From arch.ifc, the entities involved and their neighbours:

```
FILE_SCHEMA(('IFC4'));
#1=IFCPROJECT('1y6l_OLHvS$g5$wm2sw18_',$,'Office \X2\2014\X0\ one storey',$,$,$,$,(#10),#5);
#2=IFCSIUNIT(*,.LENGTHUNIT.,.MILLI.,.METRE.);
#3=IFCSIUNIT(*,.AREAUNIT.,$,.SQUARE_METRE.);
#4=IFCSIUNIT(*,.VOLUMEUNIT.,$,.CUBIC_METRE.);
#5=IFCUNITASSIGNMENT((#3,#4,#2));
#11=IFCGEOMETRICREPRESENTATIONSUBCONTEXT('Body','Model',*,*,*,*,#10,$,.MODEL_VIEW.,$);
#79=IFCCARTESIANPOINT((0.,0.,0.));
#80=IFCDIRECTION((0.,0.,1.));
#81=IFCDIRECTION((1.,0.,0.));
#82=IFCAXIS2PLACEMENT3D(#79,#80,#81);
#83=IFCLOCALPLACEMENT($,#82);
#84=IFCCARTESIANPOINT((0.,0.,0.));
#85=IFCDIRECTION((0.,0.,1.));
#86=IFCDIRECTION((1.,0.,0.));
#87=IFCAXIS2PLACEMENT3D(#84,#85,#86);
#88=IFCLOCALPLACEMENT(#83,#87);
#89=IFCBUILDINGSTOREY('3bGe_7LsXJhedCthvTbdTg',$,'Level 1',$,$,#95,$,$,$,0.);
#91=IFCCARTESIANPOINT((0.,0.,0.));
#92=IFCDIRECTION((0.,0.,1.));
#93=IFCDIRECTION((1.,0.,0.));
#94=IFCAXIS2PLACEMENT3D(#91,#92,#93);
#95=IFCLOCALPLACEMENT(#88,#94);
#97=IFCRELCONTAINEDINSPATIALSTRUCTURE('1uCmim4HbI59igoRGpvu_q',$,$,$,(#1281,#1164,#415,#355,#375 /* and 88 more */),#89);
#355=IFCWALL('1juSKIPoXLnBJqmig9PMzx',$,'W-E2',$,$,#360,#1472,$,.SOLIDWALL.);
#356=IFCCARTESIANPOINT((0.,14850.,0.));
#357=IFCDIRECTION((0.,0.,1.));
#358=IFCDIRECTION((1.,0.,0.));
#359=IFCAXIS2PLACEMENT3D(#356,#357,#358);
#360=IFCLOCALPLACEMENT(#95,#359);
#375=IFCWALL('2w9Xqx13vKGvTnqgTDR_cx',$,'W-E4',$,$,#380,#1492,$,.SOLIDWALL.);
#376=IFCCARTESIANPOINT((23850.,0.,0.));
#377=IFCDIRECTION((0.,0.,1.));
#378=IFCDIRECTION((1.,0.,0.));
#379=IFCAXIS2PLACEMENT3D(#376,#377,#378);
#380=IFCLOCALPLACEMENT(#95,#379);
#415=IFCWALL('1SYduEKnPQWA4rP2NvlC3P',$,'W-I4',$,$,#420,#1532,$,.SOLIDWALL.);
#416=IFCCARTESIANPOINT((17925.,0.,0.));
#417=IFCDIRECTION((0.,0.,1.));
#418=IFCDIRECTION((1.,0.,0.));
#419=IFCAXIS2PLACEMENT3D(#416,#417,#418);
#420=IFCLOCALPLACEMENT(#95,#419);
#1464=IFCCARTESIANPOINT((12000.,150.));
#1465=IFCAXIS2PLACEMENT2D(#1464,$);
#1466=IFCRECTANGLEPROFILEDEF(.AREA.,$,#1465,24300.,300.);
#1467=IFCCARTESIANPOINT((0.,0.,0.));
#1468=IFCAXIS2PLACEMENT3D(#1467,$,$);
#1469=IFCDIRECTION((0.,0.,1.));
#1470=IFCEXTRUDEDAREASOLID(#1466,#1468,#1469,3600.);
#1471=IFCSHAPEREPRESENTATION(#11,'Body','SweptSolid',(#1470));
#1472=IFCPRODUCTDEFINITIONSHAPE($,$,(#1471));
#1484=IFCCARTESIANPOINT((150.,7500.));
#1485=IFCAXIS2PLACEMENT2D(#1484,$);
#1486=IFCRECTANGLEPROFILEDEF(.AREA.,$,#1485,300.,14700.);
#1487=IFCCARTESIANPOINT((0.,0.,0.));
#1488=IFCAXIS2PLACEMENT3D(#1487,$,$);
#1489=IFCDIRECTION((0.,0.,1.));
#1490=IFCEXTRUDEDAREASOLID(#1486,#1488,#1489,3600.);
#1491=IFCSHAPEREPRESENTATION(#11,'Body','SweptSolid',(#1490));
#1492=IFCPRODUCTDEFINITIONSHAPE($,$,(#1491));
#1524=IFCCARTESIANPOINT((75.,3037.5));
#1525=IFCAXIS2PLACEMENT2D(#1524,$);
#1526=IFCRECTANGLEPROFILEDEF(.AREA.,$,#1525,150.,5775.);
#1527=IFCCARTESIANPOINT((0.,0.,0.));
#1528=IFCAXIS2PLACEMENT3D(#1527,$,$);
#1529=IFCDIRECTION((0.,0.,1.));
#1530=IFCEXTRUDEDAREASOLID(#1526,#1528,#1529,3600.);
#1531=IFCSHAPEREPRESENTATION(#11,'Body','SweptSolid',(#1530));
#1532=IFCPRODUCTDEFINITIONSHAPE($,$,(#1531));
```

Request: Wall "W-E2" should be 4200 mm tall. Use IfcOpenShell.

```python
import ifcopenshell
import ifcopenshell.geom
import ifcopenshell.util.representation
import ifcopenshell.util.shape
import ifcopenshell.util.unit

model = ifcopenshell.open("arch.ifc")
unit_scale = ifcopenshell.util.unit.calculate_unit_scale(model)
settings = ifcopenshell.geom.settings()


def volume(element):
    """Net volume in cubic metres, openings subtracted."""
    shape = ifcopenshell.geom.create_shape(settings, element)
    return ifcopenshell.util.shape.get_volume(shape.geometry)


wall = model.by_guid("1juSKIPoXLnBJqmig9PMzx")
before = volume(wall)

body = ifcopenshell.util.representation.get_representation(wall, "Model", "Body")
solid = body.Items[0]
old_height = solid.Depth
solid.Depth = 4.2 / unit_scale
after = volume(wall)

print(f"height {old_height:g} -> {solid.Depth:g}, volume {before:.3f} -> {after:.3f} m3")

model.write("arch-out.ifc")
```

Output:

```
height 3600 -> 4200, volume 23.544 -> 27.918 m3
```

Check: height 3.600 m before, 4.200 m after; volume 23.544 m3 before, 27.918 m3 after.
